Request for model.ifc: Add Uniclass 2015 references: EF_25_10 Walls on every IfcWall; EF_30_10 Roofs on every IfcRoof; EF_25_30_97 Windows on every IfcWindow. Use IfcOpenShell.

First a look at what the model holds.

```python
import ifcopenshell

model = ifcopenshell.open("model.ifc")
print(model.schema)
print("classifications:", [c.Name for c in model.by_type("IfcClassification")])
for ifc_class in ("IfcDoor", "IfcRoof", "IfcStair", "IfcWall", "IfcWindow"):
    print(ifc_class, len(model.by_type(ifc_class)))
```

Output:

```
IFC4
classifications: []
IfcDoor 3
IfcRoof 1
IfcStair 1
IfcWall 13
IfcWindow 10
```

```python
import ifcopenshell
import ifcopenshell.api.classification

model = ifcopenshell.open("model.ifc")

system = ifcopenshell.api.classification.add_classification(model, classification="Uniclass 2015")

codes = {
    "IfcWall": ("EF_25_10", "Walls"),
    "IfcRoof": ("EF_30_10", "Roofs"),
    "IfcWindow": ("EF_25_30_97", "Windows"),
}
for ifc_class, (code, name) in codes.items():
    products = model.by_type(ifc_class)
    ifcopenshell.api.classification.add_reference(
        model, products=products, classification=system, identification=code, name=name
    )
    print(code, len(products))

model.write("model_v2.ifc")
```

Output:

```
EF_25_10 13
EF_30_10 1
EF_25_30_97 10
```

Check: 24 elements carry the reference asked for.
